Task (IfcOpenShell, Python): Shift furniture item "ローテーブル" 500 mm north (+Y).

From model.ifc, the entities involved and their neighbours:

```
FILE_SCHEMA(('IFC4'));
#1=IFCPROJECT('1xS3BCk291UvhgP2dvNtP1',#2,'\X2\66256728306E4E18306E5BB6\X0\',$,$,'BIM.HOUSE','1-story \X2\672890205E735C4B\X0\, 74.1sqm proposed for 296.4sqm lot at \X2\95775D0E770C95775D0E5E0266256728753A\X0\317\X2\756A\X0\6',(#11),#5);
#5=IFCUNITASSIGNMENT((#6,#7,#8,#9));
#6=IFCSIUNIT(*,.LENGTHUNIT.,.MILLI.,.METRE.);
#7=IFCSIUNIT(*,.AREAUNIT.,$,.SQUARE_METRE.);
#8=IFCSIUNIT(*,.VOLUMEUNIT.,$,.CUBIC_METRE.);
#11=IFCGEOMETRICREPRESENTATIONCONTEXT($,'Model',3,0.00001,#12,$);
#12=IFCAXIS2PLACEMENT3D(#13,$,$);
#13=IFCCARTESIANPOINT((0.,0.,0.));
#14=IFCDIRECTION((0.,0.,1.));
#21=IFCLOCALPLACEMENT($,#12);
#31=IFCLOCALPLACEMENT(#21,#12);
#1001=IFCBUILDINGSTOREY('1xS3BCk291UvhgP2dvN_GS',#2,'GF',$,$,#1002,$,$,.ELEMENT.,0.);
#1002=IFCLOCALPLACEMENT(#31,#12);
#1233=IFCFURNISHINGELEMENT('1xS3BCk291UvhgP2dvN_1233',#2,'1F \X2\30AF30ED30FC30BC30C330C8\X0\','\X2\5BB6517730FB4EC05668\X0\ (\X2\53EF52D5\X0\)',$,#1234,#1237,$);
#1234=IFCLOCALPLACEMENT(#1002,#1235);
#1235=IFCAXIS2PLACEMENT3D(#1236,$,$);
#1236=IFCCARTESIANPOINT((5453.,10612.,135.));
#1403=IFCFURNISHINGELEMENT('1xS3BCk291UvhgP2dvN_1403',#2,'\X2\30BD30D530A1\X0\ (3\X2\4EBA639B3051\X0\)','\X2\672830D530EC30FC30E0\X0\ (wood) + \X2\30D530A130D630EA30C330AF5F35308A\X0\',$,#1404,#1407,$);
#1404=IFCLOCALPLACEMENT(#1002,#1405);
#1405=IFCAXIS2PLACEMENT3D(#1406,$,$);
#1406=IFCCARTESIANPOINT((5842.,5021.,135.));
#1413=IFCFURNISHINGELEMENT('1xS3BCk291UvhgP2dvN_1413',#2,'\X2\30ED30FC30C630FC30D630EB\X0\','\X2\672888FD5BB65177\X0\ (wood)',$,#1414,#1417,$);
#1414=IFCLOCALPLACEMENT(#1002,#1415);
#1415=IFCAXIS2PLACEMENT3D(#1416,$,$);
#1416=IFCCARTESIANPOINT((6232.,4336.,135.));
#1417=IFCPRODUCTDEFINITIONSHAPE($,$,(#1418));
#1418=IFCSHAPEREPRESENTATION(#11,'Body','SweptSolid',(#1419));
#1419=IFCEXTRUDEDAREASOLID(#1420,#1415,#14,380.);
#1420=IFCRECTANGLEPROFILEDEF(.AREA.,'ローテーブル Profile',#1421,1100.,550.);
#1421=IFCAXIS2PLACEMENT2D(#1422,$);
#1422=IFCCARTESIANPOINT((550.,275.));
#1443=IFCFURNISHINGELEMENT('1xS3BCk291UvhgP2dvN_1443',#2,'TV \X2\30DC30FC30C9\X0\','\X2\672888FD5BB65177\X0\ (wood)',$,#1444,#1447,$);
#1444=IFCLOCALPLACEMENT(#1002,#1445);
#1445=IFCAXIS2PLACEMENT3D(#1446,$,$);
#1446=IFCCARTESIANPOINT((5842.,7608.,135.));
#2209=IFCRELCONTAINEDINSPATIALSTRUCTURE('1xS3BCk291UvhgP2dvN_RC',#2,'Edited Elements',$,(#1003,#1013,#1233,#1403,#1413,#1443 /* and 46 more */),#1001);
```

```python
import ifcopenshell
import ifcopenshell.api.geometry
import ifcopenshell.util.placement
import ifcopenshell.util.unit

model = ifcopenshell.open("model.ifc")
unit_scale = ifcopenshell.util.unit.calculate_unit_scale(model)

item = model.by_id(1413)
matrix = ifcopenshell.util.placement.get_local_placement(item.ObjectPlacement)
matrix[1, 3] += 0.5 / unit_scale
ifcopenshell.api.geometry.edit_object_placement(model, product=item, matrix=matrix, is_si=False)

print(ifcopenshell.util.placement.get_local_placement(item.ObjectPlacement).round(3) + 0.0)

model.write("model_edited.ifc")
```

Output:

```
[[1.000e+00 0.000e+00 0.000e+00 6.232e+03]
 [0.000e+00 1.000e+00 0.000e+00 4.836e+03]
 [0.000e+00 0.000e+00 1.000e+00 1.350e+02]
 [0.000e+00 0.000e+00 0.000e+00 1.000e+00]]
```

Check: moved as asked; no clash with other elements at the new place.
